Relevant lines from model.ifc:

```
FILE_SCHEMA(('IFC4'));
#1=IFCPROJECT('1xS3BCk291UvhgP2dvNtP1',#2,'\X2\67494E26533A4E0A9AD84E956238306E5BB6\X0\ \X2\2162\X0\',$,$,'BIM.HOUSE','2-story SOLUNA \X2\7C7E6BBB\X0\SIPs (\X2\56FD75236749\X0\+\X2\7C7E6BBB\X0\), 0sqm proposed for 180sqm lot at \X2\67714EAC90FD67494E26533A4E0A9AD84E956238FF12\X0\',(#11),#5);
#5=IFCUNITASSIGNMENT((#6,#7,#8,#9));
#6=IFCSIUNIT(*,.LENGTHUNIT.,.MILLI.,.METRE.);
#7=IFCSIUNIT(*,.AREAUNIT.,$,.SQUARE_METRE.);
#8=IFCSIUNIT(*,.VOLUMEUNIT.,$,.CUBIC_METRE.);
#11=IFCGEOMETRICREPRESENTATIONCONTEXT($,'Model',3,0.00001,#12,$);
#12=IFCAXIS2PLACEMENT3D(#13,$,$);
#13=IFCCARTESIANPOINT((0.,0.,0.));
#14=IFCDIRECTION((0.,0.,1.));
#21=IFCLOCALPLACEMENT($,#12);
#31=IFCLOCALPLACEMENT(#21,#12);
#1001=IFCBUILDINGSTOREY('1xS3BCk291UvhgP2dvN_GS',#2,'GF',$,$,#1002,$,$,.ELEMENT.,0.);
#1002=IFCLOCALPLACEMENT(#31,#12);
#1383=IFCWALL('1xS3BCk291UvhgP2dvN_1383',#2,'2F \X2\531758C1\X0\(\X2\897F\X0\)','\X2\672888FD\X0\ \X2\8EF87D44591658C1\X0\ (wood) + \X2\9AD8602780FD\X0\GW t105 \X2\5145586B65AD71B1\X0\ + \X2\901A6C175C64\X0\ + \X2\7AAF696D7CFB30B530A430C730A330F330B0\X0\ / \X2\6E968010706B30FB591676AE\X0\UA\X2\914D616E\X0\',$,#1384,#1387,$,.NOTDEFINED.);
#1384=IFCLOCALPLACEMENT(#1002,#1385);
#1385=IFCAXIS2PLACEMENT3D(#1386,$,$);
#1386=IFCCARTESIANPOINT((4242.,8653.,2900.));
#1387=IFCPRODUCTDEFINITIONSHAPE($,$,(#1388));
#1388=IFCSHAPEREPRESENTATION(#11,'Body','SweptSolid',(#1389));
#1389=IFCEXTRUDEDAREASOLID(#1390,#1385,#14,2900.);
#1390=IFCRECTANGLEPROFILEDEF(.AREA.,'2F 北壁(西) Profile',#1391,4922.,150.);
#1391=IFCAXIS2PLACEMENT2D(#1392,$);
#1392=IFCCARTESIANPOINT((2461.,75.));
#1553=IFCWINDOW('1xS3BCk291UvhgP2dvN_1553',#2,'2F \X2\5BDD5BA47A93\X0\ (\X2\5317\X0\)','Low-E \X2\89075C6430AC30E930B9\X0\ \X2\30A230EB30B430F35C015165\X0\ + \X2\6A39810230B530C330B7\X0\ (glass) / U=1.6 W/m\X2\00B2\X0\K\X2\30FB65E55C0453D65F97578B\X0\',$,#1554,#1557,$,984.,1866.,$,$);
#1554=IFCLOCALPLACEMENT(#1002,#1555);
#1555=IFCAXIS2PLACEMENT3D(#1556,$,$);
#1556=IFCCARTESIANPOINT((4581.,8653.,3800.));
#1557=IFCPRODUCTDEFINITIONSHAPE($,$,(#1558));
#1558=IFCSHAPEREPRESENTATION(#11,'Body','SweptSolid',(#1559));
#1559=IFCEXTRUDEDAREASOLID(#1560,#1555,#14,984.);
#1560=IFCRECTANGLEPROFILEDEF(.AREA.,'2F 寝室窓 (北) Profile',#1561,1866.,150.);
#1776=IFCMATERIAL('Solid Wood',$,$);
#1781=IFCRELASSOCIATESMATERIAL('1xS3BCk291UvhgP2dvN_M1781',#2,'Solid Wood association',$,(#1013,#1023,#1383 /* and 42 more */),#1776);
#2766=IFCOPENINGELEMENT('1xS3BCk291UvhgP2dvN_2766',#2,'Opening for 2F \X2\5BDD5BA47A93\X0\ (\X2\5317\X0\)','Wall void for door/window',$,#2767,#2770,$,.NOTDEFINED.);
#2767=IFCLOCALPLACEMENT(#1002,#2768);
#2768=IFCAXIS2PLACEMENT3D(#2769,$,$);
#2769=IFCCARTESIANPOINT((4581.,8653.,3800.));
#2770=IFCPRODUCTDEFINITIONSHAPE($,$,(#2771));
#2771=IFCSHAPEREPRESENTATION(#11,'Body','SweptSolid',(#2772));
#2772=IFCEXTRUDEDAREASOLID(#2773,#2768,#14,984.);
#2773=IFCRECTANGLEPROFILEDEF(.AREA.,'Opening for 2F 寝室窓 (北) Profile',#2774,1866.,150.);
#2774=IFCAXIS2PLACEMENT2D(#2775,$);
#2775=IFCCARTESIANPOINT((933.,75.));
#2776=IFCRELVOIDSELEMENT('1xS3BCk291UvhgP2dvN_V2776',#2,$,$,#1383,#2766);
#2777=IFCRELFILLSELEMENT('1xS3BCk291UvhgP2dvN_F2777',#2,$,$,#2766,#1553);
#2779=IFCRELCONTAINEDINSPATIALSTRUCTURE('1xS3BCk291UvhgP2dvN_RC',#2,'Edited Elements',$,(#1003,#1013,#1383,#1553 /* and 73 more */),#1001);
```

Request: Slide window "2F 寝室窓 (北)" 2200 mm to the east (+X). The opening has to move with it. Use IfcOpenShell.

```python
import ifcopenshell
import ifcopenshell.api.geometry
import ifcopenshell.util.placement
import ifcopenshell.util.unit

model = ifcopenshell.open("model.ifc")
unit_scale = ifcopenshell.util.unit.calculate_unit_scale(model)

window = model.by_guid("1xS3BCk291UvhgP2dvN_1553")
opening = window.FillsVoids[0].RelatingOpeningElement
wall = opening.VoidsElements[0].RelatingBuildingElement

wall_matrix = ifcopenshell.util.placement.get_local_placement(wall.ObjectPlacement)
shift = wall_matrix[:3, 0] * 2.2 / unit_scale
before = ifcopenshell.util.placement.get_local_placement(window.ObjectPlacement)[:3, 3].copy()

# The window is not placed relative to its opening, so move both.
for product in (opening, window):
    matrix = ifcopenshell.util.placement.get_local_placement(product.ObjectPlacement)
    matrix[:3, 3] += shift
    ifcopenshell.api.geometry.edit_object_placement(model, product=product, matrix=matrix, is_si=False)

after = ifcopenshell.util.placement.get_local_placement(window.ObjectPlacement)[:3, 3]
print("window moved by", (after - before).round(3) + 0.0)

model.write("model_rev.ifc")
```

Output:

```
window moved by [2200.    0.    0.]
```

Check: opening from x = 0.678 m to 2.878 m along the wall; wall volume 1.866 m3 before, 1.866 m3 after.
